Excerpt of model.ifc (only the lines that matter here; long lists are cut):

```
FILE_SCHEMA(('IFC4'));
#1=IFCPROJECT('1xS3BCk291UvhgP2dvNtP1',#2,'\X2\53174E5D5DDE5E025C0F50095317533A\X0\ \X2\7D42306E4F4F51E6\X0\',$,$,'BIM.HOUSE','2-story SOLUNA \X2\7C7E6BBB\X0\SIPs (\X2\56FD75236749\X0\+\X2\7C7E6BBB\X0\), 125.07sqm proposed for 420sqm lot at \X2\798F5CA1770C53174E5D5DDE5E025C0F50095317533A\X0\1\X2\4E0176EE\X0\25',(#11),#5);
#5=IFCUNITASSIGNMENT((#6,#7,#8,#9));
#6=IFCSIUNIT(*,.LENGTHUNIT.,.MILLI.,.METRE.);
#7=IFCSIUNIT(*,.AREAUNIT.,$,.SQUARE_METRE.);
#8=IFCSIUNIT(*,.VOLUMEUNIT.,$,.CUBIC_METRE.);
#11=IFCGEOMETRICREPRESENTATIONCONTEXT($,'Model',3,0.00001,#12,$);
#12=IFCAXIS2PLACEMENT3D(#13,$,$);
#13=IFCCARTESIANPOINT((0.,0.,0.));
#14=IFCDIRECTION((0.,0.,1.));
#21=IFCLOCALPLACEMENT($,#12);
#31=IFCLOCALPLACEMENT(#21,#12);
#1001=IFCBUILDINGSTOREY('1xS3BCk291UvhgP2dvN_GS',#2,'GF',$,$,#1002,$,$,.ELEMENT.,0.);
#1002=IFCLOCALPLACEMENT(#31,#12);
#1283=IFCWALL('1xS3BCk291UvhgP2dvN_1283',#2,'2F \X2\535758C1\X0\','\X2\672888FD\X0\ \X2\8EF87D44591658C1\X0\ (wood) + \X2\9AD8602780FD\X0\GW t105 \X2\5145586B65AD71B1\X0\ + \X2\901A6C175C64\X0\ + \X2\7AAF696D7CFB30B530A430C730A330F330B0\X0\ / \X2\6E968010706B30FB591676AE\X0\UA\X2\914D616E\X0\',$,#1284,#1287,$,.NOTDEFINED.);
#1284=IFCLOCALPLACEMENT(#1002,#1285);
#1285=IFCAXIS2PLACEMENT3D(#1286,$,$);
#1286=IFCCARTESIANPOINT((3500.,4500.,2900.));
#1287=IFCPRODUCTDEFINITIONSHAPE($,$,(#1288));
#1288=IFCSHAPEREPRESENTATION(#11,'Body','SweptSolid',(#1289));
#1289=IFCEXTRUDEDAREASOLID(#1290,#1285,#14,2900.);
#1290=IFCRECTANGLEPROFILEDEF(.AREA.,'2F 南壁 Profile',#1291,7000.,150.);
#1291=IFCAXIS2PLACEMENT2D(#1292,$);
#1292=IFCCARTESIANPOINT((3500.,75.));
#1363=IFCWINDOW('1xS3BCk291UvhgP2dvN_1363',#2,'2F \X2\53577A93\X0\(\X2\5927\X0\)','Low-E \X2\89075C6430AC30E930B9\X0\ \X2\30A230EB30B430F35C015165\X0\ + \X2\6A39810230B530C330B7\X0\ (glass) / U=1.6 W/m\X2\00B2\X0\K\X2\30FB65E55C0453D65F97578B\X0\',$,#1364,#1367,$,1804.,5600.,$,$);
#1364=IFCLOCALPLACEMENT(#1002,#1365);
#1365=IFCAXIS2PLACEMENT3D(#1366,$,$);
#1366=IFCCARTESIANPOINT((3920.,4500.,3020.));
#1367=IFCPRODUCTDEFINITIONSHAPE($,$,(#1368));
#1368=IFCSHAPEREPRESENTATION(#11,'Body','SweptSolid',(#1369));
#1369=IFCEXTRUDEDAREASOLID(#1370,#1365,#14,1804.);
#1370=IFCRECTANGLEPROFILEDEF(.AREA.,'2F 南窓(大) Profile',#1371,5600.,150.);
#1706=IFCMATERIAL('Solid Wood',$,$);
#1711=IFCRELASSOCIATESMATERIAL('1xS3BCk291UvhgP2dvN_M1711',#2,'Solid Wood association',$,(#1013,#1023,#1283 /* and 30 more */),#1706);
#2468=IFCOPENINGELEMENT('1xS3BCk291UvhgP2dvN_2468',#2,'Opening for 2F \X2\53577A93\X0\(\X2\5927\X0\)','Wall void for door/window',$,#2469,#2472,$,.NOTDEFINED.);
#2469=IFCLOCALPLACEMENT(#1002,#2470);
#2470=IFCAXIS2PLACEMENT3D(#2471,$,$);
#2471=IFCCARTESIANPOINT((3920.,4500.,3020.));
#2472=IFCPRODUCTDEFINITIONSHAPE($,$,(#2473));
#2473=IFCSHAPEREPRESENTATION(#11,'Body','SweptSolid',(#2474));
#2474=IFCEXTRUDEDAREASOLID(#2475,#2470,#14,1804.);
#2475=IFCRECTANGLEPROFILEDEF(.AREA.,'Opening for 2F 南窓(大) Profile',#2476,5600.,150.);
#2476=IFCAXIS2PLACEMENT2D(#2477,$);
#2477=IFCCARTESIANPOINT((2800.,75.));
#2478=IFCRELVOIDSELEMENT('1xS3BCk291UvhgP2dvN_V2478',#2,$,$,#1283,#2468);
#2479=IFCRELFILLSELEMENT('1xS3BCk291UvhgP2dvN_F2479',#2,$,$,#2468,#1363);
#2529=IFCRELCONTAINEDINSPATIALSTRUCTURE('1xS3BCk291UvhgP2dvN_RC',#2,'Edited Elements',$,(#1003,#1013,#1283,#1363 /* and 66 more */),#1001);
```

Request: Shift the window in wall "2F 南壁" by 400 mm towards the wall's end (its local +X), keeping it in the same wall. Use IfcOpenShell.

```python
import ifcopenshell
import ifcopenshell.api.geometry
import ifcopenshell.util.placement

model = ifcopenshell.open("model.ifc")

window = model.by_id(1363)
opening = window.FillsVoids[0].RelatingOpeningElement
wall = opening.VoidsElements[0].RelatingBuildingElement

wall_matrix = ifcopenshell.util.placement.get_local_placement(wall.ObjectPlacement)
shift = wall_matrix[:3, 0] * 400.0
before = ifcopenshell.util.placement.get_local_placement(window.ObjectPlacement)[:3, 3].copy()

# The window is not placed relative to its opening, so move both.
for product in (opening, window):
    matrix = ifcopenshell.util.placement.get_local_placement(product.ObjectPlacement)
    matrix[:3, 3] += shift
    ifcopenshell.api.geometry.edit_object_placement(model, product=product, matrix=matrix, is_si=False)

after = ifcopenshell.util.placement.get_local_placement(window.ObjectPlacement)[:3, 3]
print("window moved by", (after - before).round(3) + 0.0)

model.write("model_updated.ifc")
```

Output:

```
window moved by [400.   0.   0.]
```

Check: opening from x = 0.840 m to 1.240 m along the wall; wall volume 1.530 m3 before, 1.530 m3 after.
